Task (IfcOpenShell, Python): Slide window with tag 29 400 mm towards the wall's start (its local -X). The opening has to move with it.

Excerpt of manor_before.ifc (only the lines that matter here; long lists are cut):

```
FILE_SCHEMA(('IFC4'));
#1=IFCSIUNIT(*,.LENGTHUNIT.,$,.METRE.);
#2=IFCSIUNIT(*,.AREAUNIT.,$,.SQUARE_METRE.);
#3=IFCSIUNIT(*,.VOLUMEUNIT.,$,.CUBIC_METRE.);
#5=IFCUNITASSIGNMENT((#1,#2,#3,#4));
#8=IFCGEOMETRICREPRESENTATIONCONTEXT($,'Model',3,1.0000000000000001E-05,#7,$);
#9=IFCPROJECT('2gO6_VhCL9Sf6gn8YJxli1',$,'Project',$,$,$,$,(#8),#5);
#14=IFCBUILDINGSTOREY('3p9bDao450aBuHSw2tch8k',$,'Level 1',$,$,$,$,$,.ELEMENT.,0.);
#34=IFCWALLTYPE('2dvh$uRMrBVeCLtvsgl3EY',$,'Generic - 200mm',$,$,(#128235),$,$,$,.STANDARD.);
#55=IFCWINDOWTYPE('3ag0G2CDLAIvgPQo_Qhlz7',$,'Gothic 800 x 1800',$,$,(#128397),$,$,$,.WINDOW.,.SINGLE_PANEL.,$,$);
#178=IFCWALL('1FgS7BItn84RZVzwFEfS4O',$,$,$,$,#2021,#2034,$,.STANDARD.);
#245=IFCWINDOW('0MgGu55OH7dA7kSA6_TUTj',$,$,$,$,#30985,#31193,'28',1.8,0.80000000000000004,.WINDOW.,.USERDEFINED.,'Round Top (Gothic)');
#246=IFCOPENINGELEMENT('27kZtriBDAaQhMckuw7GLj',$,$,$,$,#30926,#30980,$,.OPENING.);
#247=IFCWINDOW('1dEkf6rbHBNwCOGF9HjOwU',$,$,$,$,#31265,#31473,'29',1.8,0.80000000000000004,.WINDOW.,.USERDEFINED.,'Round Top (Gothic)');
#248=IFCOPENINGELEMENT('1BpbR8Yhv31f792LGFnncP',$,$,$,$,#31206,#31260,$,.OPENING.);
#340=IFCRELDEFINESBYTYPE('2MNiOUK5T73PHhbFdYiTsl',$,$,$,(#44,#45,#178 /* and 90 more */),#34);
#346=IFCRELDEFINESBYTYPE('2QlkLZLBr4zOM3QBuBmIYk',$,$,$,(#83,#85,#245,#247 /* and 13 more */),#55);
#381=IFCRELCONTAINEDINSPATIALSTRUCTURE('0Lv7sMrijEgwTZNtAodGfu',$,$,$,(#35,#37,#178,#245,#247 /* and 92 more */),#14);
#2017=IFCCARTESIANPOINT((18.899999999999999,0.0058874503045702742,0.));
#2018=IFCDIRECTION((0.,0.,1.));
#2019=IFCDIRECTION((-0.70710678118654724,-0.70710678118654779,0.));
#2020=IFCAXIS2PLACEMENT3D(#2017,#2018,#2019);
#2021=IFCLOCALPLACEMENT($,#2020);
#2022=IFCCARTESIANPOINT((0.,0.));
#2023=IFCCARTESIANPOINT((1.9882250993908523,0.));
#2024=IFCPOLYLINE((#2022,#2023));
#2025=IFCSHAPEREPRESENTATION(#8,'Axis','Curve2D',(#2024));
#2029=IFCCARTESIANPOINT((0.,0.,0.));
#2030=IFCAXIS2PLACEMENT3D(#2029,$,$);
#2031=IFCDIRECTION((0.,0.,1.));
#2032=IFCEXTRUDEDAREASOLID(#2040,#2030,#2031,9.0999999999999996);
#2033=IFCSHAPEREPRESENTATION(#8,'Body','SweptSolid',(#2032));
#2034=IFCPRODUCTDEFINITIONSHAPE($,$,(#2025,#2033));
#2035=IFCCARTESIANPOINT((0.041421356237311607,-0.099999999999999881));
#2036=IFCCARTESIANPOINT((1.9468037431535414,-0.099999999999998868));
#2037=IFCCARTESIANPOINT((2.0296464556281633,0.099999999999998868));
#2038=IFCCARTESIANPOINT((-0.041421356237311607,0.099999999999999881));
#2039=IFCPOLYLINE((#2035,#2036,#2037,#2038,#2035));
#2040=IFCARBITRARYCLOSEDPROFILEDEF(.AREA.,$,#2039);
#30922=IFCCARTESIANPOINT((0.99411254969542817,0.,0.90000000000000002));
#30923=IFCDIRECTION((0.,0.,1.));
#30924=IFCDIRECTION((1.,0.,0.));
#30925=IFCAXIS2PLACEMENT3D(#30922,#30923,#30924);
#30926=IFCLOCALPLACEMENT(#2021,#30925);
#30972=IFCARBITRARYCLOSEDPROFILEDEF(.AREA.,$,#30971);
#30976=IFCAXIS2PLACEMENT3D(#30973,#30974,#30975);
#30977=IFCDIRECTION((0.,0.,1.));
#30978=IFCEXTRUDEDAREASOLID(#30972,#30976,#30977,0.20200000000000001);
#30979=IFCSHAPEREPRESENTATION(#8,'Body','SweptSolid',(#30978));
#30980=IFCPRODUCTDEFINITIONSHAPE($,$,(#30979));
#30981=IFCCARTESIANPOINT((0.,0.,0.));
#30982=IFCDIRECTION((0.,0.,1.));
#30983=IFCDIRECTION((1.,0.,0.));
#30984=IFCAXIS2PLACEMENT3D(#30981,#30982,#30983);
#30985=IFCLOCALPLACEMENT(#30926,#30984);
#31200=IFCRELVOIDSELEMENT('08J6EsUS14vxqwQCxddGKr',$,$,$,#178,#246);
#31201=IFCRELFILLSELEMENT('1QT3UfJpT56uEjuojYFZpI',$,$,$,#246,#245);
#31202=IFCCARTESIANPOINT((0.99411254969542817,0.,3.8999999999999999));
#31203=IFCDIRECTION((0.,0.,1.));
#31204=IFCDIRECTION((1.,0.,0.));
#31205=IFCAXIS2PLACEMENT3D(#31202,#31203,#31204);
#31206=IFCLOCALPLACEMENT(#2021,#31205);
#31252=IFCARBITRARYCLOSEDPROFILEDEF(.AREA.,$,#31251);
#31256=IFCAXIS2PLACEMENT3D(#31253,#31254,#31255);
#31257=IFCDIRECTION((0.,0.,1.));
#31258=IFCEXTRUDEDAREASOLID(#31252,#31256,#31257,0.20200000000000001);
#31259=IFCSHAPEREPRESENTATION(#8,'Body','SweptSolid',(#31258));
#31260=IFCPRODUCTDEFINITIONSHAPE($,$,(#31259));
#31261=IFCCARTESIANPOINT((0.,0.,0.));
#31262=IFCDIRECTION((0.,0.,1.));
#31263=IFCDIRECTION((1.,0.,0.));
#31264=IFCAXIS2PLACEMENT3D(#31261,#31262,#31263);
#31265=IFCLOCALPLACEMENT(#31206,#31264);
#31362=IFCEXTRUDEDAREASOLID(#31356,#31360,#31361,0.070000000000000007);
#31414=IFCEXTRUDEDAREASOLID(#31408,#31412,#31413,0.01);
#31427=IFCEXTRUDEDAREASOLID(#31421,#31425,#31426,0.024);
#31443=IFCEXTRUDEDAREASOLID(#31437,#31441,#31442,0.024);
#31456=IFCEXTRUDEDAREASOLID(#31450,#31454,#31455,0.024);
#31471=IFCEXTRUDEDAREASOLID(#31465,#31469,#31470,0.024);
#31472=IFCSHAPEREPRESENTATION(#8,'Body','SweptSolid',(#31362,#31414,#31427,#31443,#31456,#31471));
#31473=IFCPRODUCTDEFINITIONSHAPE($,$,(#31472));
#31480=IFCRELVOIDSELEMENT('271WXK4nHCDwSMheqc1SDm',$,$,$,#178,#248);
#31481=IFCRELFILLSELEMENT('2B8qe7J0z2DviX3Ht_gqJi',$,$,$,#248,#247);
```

```python
import ifcopenshell
import ifcopenshell.api.geometry
import ifcopenshell.util.placement

model = ifcopenshell.open("manor_before.ifc")

window = model.by_id(247)
opening = window.FillsVoids[0].RelatingOpeningElement
wall = opening.VoidsElements[0].RelatingBuildingElement

wall_matrix = ifcopenshell.util.placement.get_local_placement(wall.ObjectPlacement)
shift = wall_matrix[:3, 0] * -0.4
before = ifcopenshell.util.placement.get_local_placement(window.ObjectPlacement)[:3, 3].copy()

# The window is placed relative to its opening, so it follows when the opening moves.
matrix = ifcopenshell.util.placement.get_local_placement(opening.ObjectPlacement)
matrix[:3, 3] += shift
ifcopenshell.api.geometry.edit_object_placement(
    model, product=opening, matrix=matrix, is_si=False, should_transform_children=True
)

after = ifcopenshell.util.placement.get_local_placement(window.ObjectPlacement)[:3, 3]
print("window moved by", (after - before).round(3) + 0.0)

model.write("manor_before-out.ifc")
```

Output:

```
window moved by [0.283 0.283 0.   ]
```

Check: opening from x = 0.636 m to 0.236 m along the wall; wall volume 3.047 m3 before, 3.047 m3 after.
